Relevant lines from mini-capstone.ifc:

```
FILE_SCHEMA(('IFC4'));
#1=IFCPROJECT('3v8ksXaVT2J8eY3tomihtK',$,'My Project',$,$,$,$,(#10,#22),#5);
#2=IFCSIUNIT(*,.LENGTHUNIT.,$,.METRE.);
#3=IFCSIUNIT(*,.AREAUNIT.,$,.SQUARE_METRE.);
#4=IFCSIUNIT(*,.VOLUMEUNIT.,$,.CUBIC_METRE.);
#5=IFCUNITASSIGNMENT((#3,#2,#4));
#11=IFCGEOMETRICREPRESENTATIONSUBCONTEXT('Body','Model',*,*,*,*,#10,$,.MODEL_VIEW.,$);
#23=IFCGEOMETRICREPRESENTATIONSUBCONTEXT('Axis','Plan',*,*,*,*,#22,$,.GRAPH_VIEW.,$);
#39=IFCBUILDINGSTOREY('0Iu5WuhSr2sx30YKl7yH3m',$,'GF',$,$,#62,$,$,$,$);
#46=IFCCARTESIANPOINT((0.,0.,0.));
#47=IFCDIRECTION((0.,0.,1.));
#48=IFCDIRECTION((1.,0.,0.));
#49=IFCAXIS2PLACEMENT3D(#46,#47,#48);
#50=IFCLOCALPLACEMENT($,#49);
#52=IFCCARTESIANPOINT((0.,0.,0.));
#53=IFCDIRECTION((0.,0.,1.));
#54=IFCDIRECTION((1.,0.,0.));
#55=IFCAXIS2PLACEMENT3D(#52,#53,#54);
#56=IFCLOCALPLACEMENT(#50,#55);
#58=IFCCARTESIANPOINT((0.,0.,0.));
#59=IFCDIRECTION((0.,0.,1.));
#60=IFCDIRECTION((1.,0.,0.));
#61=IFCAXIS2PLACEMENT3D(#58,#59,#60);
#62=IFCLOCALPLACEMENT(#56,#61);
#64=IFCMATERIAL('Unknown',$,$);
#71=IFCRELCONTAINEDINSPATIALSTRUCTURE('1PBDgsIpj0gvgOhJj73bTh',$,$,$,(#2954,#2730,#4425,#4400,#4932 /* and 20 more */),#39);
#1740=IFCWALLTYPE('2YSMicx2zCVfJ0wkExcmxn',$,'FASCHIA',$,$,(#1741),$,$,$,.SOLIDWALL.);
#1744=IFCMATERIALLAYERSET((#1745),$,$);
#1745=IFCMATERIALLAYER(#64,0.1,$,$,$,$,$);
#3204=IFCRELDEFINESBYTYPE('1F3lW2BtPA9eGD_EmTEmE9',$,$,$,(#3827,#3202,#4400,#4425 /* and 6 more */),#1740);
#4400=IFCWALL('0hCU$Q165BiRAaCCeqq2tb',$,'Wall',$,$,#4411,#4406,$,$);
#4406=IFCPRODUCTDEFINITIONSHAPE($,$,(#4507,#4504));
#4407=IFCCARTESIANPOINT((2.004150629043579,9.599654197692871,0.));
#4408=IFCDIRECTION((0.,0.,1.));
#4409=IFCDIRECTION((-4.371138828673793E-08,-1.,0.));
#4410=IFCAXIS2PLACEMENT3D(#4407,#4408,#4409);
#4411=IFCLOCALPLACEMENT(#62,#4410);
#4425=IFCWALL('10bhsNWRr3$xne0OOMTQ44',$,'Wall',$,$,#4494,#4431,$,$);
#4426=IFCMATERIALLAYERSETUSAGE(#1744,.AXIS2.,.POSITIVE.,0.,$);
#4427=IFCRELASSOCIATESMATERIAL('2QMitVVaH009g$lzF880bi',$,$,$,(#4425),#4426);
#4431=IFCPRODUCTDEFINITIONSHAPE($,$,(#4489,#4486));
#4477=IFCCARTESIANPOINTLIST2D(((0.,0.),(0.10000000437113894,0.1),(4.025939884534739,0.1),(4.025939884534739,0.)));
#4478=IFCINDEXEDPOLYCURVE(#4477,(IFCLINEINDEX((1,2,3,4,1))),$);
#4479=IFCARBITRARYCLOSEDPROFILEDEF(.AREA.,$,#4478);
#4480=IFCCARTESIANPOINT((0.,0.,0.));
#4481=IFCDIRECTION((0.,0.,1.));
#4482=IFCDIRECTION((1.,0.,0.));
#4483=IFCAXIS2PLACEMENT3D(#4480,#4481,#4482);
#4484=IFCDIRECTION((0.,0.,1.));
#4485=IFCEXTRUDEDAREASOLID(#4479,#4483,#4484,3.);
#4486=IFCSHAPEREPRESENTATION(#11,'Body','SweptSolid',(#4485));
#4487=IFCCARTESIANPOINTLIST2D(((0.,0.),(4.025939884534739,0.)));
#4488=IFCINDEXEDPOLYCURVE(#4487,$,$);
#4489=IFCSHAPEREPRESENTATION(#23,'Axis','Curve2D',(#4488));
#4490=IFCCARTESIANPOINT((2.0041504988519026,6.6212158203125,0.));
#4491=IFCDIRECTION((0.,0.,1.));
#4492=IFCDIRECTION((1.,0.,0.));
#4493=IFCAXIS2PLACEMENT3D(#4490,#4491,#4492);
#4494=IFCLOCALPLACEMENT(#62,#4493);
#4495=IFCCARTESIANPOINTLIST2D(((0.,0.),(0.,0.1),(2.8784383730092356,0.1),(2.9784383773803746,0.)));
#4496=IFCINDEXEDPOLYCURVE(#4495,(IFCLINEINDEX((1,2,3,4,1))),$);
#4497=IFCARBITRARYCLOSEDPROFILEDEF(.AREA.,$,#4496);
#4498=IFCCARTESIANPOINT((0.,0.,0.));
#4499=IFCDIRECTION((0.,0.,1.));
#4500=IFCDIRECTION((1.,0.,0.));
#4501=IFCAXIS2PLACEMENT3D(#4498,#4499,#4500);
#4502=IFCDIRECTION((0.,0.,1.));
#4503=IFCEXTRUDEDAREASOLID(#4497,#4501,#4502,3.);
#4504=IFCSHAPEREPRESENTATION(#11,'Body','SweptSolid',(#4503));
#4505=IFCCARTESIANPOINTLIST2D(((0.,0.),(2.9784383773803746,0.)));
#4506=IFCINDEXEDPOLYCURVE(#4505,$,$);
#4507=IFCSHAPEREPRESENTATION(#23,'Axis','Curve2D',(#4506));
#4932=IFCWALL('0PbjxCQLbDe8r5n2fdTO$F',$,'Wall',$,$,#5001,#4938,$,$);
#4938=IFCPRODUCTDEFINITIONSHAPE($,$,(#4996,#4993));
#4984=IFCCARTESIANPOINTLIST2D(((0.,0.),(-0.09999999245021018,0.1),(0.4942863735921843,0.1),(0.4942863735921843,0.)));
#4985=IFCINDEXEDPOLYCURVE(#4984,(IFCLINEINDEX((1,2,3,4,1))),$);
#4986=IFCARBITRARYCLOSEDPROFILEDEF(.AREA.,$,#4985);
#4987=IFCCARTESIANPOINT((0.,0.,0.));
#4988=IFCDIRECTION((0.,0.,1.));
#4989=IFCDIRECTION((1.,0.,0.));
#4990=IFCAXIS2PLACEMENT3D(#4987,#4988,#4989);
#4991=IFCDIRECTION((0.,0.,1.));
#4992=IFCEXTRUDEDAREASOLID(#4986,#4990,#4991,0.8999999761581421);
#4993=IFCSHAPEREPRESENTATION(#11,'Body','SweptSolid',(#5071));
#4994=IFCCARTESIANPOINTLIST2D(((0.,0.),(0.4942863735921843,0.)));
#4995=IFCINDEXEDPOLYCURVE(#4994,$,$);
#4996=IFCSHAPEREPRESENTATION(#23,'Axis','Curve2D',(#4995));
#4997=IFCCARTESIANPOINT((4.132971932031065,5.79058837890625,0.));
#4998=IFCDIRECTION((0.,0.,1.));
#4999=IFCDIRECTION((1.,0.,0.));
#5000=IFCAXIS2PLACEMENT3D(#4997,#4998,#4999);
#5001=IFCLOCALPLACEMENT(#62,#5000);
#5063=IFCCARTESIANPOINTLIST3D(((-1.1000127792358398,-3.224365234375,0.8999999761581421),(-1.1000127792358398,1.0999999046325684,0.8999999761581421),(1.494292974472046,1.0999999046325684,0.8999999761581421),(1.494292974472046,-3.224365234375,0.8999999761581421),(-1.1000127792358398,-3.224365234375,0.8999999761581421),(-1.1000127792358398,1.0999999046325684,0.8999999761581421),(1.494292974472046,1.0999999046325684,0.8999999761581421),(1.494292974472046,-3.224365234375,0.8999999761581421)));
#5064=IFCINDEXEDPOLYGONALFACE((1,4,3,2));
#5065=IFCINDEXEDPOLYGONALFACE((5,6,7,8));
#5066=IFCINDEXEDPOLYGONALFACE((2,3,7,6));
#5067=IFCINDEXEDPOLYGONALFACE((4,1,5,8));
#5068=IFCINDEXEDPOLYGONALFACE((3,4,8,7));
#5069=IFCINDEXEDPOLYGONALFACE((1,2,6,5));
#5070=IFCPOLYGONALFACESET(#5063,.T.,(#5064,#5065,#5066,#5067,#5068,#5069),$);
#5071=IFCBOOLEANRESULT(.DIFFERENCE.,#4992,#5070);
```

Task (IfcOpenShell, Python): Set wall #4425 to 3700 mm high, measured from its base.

```python
import ifcopenshell
import ifcopenshell.geom
import ifcopenshell.util.representation
import ifcopenshell.util.shape
import ifcopenshell.util.unit

model = ifcopenshell.open("mini-capstone.ifc")
unit_scale = ifcopenshell.util.unit.calculate_unit_scale(model)
settings = ifcopenshell.geom.settings()


def volume(element):
    """Net volume in cubic metres, openings subtracted."""
    shape = ifcopenshell.geom.create_shape(settings, element)
    return ifcopenshell.util.shape.get_volume(shape.geometry)


wall = model.by_guid("10bhsNWRr3$xne0OOMTQ44")
before = volume(wall)

body = ifcopenshell.util.representation.get_representation(wall, "Model", "Body")
solid = body.Items[0]
old_height = solid.Depth
solid.Depth = 3.7 / unit_scale
after = volume(wall)

print(f"height {old_height:g} -> {solid.Depth:g}, volume {before:.3f} -> {after:.3f} m3")

model.write("mini-capstone_edited.ifc")
```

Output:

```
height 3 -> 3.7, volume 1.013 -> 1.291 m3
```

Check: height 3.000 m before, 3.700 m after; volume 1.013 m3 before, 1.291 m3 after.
